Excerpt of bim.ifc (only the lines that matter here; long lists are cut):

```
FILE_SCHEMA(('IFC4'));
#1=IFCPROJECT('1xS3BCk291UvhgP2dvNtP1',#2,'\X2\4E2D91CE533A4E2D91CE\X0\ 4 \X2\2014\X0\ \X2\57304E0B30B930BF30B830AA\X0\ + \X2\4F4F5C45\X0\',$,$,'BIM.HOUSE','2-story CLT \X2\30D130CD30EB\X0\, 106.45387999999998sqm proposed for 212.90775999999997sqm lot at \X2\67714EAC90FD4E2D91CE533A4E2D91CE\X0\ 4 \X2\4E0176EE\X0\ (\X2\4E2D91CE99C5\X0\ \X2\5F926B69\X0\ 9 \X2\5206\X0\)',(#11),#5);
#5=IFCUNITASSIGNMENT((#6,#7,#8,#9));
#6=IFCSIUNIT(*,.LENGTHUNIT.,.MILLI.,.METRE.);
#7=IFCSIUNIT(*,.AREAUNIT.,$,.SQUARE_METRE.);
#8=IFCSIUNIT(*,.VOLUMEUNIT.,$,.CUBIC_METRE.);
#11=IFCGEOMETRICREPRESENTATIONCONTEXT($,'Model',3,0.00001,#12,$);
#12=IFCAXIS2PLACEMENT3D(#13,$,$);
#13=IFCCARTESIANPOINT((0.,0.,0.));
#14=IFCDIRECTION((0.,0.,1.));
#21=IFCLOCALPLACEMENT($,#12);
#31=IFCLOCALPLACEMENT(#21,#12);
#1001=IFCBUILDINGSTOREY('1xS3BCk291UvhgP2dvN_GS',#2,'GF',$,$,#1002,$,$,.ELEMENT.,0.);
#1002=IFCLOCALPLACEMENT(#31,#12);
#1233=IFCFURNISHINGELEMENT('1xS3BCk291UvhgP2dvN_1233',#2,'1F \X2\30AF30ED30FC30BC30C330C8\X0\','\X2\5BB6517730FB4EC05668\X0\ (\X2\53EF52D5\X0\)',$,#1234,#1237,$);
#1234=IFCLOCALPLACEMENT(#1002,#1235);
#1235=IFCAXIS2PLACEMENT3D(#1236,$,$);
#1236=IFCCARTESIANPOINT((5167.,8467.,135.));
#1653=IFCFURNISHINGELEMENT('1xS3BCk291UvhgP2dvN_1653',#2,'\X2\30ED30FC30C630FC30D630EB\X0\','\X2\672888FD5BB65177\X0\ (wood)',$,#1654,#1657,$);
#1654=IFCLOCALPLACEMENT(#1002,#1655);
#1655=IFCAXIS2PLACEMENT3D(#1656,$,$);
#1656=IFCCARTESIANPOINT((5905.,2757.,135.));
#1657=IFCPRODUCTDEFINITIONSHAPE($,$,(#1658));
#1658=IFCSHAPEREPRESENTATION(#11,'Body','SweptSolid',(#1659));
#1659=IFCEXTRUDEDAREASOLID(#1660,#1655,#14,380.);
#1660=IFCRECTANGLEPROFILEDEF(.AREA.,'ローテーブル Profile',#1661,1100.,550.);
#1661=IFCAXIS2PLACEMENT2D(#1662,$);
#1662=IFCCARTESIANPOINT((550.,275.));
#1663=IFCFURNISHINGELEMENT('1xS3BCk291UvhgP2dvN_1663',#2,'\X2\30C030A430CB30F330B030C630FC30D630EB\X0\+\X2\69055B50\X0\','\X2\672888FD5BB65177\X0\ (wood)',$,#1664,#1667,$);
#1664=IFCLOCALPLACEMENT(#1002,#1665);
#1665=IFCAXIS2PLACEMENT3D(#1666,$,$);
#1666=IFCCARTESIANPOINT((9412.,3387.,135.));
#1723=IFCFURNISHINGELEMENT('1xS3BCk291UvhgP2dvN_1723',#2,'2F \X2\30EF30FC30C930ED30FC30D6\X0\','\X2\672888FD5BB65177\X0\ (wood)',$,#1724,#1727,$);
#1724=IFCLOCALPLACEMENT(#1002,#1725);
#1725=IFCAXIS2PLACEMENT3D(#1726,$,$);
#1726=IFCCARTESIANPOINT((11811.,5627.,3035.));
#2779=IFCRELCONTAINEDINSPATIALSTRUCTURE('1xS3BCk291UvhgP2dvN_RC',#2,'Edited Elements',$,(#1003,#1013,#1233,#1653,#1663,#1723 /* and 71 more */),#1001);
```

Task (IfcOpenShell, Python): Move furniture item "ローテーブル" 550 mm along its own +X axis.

```python
import ifcopenshell
import ifcopenshell.api.geometry
import ifcopenshell.util.placement

model = ifcopenshell.open("bim.ifc")

item = model.by_guid("1xS3BCk291UvhgP2dvN_1653")
matrix = ifcopenshell.util.placement.get_local_placement(item.ObjectPlacement)
matrix[:3, 3] += matrix[:3, 0] * 550.0
ifcopenshell.api.geometry.edit_object_placement(model, product=item, matrix=matrix, is_si=False)

print(ifcopenshell.util.placement.get_local_placement(item.ObjectPlacement).round(3) + 0.0)

model.write("bim_edited.ifc")
```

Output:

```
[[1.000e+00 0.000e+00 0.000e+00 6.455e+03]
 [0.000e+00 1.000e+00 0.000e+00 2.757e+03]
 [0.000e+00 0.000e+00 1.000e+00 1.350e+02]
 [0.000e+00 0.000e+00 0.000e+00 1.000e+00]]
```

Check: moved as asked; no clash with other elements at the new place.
